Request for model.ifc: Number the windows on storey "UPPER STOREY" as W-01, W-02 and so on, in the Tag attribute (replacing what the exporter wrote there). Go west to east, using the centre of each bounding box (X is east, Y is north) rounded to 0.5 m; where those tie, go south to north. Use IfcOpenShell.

First a look at what the model holds.

```python
import ifcopenshell
import ifcopenshell.util.element
import ifcopenshell.util.placement

model = ifcopenshell.open("model.ifc")
print(model.schema)
storey = next(s for s in model.by_type("IfcBuildingStorey") if s.Name == "UPPER STOREY")
windows = [e for e in ifcopenshell.util.element.get_decomposition(storey) if e.is_a("IfcWindow")]
for e in sorted(windows, key=lambda e: e.id()):
    origin = ifcopenshell.util.placement.get_local_placement(e.ObjectPlacement)[:3, 3]
    print(e.id(), e.Tag, e.Name, origin.round(2) + 0.0, sep=" | ")
```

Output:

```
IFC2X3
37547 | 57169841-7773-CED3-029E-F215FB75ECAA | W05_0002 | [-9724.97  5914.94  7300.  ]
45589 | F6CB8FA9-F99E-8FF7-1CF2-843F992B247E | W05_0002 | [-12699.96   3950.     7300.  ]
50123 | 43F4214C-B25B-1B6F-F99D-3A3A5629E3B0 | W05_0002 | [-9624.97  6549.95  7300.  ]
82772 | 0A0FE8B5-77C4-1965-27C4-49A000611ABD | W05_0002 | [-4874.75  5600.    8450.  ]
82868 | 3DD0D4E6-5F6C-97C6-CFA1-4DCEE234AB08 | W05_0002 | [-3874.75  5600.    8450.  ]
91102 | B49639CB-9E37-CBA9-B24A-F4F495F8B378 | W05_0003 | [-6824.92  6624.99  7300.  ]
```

```python
import ifcopenshell
import ifcopenshell.geom
import ifcopenshell.util.element
import ifcopenshell.util.shape

model = ifcopenshell.open("model.ifc")
settings = ifcopenshell.geom.settings()
settings.set("use-world-coords", True)


def centre(element):
    shape = ifcopenshell.geom.create_shape(settings, element)
    return ifcopenshell.util.shape.get_bbox_centroid(shape.geometry)


storey = next(s for s in model.by_type("IfcBuildingStorey") if s.Name == "UPPER STOREY")
windows = [e for e in ifcopenshell.util.element.get_decomposition(storey) if e.is_a("IfcWindow")]

# Insertion points can sit at a corner or the storey origin, so sort by the geometry (in metres).
centres = {e: centre(e) for e in windows}
windows.sort(key=lambda e: (round(centres[e][0] / 0.5), centres[e][1]))

for i, e in enumerate(windows, start=1):
    number = f"W-{i:02d}"
    e.Tag = number
    print(e.id(), number)

model.write("model_v2.ifc")
```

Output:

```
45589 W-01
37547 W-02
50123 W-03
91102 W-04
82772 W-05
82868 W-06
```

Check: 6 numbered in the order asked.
